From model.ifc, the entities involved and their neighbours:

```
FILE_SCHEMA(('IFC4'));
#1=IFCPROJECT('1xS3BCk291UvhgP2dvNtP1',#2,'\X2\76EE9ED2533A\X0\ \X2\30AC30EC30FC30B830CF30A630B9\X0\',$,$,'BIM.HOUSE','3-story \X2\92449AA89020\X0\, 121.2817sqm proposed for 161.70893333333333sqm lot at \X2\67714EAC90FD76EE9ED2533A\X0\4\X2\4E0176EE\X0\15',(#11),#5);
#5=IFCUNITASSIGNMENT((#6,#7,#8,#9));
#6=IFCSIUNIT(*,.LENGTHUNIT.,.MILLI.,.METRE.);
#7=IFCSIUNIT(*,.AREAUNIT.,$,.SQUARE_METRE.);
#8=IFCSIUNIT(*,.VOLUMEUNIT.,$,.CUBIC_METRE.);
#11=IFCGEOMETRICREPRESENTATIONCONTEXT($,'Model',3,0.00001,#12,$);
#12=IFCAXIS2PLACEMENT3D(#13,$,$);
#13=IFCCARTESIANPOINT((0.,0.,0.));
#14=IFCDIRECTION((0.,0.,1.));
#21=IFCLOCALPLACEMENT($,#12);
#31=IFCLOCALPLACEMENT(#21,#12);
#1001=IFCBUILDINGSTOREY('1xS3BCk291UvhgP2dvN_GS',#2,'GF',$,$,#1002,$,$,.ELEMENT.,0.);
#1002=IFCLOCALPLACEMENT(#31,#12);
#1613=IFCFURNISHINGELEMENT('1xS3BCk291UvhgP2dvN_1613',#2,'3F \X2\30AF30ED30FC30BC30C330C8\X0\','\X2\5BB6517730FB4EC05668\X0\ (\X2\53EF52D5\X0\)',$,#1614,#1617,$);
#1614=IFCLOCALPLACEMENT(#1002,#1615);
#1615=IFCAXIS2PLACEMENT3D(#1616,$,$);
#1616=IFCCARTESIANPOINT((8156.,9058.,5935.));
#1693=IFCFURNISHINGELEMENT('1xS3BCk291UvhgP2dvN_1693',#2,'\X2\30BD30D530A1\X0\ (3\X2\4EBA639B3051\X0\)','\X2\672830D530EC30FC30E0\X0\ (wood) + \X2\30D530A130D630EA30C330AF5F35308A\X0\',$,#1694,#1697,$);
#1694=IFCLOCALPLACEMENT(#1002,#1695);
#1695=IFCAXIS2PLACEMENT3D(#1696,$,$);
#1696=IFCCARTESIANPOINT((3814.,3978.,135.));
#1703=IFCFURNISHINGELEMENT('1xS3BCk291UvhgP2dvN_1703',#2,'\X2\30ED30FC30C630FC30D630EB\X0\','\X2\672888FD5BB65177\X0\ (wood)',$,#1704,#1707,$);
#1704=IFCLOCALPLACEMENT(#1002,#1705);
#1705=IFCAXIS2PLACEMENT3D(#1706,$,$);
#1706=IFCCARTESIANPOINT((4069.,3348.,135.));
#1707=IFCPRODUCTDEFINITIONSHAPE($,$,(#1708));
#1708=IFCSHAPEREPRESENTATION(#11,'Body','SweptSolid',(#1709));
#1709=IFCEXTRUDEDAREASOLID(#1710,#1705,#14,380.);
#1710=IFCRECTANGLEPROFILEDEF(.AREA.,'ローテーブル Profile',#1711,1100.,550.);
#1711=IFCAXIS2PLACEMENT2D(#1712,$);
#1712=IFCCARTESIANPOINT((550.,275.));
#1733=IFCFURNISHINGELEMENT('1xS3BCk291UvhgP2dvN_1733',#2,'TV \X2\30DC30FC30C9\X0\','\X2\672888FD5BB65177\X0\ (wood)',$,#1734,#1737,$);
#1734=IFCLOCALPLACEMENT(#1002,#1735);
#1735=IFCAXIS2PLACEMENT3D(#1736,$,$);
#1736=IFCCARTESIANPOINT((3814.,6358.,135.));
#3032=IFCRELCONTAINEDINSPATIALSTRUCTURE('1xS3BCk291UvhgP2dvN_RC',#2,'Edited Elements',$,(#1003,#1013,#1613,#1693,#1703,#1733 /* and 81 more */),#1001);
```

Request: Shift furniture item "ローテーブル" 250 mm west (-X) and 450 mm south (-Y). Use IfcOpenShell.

```python
import ifcopenshell
import ifcopenshell.api.geometry
import ifcopenshell.util.placement

model = ifcopenshell.open("model.ifc")

item = model.by_guid("1xS3BCk291UvhgP2dvN_1703")
matrix = ifcopenshell.util.placement.get_local_placement(item.ObjectPlacement)
matrix[0, 3] -= 250.0
matrix[1, 3] -= 450.0
ifcopenshell.api.geometry.edit_object_placement(model, product=item, matrix=matrix, is_si=False)

print(ifcopenshell.util.placement.get_local_placement(item.ObjectPlacement).round(3) + 0.0)

model.write("model_edited.ifc")
```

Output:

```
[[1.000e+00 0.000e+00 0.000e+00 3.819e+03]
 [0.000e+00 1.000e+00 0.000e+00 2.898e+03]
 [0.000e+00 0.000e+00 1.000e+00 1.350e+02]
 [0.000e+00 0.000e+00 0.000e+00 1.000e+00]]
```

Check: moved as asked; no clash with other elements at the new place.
